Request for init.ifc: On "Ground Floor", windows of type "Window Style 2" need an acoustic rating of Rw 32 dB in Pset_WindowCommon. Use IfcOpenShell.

First a look at what the model holds.

```python
import ifcopenshell
import ifcopenshell.util.element

model = ifcopenshell.open("init.ifc")
print(model.schema)
storey = next(s for s in model.by_type("IfcBuildingStorey") if s.Name == "Ground Floor")
windows = [e for e in ifcopenshell.util.element.get_decomposition(storey) if e.is_a("IfcWindow")]
seen = {}
for e in windows:
    element_type = ifcopenshell.util.element.get_type(e)
    key = (element_type.Name if element_type != e and element_type else None, ifcopenshell.util.element.get_pset(e, "Pset_WindowCommon", "AcousticRating"))
    seen[key] = seen.get(key, 0) + 1
for (name, value), count in sorted(seen.items(), key=str):
    print(count, "x", name, "|", value)
```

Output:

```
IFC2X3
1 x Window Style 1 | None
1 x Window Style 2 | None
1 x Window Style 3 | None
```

```python
import ifcopenshell
import ifcopenshell.api.pset
import ifcopenshell.util.element

model = ifcopenshell.open("init.ifc")

storey = next(s for s in model.by_type("IfcBuildingStorey") if s.Name == "Ground Floor")
windows = [e for e in ifcopenshell.util.element.get_decomposition(storey) if e.is_a("IfcWindow")]

count = 0
for e in windows:
    element_type = ifcopenshell.util.element.get_type(e)
    if element_type in (None, e) or element_type.Name != "Window Style 2":
        continue
    # add_pset returns the element's existing set when there is one.
    pset = ifcopenshell.api.pset.add_pset(model, product=e, name="Pset_WindowCommon")
    ifcopenshell.api.pset.edit_pset(model, pset=pset, properties={"AcousticRating": "Rw 32 dB"})
    count += 1

print(count, "windows updated")

model.write("init-out.ifc")
```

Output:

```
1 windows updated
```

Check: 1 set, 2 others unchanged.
